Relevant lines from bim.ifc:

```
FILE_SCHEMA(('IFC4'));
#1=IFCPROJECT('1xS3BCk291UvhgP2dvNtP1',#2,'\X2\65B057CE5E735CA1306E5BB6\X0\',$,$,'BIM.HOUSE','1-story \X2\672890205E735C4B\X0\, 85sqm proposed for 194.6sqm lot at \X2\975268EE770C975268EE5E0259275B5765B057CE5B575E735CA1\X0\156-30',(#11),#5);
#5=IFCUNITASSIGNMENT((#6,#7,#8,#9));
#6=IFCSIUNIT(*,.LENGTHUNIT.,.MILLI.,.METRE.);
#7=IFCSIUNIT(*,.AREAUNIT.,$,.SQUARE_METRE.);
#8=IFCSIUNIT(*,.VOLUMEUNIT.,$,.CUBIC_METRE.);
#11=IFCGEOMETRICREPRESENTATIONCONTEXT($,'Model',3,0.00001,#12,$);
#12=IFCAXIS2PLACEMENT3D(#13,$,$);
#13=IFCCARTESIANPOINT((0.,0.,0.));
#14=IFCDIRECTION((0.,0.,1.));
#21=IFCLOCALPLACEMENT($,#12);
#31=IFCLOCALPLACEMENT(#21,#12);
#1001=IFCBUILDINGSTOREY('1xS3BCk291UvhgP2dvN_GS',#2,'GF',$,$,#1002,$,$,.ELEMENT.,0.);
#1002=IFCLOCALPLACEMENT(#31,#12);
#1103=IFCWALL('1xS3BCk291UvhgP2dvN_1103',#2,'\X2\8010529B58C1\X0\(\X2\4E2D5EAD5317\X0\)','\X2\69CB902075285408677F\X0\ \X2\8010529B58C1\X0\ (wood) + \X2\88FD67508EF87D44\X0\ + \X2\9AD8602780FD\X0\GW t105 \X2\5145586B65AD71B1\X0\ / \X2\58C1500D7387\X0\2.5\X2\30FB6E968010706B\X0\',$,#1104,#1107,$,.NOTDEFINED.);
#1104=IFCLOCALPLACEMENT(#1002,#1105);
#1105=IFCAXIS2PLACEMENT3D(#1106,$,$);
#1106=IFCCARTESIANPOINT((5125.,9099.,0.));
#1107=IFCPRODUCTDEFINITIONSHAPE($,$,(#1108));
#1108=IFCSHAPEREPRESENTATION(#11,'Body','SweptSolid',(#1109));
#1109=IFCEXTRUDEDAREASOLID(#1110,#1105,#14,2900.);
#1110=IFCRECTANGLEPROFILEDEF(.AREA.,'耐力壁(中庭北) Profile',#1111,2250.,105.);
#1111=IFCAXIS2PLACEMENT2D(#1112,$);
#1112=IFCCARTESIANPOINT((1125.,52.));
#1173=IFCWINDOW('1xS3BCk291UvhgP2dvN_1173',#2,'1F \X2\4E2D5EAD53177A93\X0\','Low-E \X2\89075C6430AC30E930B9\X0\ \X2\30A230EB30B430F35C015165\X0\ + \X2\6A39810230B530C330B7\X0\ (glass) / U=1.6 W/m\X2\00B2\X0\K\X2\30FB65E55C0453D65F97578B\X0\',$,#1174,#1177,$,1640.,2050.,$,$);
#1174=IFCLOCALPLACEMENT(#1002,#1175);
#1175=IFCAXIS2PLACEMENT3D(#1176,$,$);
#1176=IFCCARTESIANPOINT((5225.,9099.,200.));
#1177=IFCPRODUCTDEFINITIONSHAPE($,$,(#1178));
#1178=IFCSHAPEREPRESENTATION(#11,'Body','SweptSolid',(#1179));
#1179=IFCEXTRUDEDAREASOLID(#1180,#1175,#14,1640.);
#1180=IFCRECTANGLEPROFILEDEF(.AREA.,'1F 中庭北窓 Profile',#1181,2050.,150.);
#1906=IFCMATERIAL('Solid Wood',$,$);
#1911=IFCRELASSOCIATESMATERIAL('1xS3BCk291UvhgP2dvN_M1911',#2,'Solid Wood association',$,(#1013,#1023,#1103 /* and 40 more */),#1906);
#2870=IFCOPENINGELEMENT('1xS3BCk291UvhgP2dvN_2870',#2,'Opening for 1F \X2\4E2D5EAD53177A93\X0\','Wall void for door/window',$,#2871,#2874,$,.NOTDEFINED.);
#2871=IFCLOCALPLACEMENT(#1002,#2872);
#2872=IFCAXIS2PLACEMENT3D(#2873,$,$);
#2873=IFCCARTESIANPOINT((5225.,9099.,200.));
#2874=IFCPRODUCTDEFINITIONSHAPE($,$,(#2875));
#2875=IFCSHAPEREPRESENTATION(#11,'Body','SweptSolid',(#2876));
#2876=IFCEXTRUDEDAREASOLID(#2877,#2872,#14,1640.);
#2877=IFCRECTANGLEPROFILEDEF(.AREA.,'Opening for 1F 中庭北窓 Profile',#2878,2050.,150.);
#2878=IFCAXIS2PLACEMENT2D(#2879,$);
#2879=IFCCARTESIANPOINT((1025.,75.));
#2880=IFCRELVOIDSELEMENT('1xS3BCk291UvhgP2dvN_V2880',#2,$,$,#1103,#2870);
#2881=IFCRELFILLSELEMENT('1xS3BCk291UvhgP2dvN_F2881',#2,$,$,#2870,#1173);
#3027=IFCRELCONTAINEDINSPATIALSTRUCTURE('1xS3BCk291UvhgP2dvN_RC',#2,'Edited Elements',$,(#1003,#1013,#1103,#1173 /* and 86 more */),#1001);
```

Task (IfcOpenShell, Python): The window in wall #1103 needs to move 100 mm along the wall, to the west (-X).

```python
import ifcopenshell
import ifcopenshell.api.geometry
import ifcopenshell.util.placement

model = ifcopenshell.open("bim.ifc")

window = model.by_guid("1xS3BCk291UvhgP2dvN_1173")
opening = window.FillsVoids[0].RelatingOpeningElement
wall = opening.VoidsElements[0].RelatingBuildingElement

wall_matrix = ifcopenshell.util.placement.get_local_placement(wall.ObjectPlacement)
shift = wall_matrix[:3, 0] * -100.0
before = ifcopenshell.util.placement.get_local_placement(window.ObjectPlacement)[:3, 3].copy()

# The window is not placed relative to its opening, so move both.
for product in (opening, window):
    matrix = ifcopenshell.util.placement.get_local_placement(product.ObjectPlacement)
    matrix[:3, 3] += shift
    ifcopenshell.api.geometry.edit_object_placement(model, product=product, matrix=matrix, is_si=False)

after = ifcopenshell.util.placement.get_local_placement(window.ObjectPlacement)[:3, 3]
print("window moved by", (after - before).round(3) + 0.0)

model.write("bim_rev.ifc")
```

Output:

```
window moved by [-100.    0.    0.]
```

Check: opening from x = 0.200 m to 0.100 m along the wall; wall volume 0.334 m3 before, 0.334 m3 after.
